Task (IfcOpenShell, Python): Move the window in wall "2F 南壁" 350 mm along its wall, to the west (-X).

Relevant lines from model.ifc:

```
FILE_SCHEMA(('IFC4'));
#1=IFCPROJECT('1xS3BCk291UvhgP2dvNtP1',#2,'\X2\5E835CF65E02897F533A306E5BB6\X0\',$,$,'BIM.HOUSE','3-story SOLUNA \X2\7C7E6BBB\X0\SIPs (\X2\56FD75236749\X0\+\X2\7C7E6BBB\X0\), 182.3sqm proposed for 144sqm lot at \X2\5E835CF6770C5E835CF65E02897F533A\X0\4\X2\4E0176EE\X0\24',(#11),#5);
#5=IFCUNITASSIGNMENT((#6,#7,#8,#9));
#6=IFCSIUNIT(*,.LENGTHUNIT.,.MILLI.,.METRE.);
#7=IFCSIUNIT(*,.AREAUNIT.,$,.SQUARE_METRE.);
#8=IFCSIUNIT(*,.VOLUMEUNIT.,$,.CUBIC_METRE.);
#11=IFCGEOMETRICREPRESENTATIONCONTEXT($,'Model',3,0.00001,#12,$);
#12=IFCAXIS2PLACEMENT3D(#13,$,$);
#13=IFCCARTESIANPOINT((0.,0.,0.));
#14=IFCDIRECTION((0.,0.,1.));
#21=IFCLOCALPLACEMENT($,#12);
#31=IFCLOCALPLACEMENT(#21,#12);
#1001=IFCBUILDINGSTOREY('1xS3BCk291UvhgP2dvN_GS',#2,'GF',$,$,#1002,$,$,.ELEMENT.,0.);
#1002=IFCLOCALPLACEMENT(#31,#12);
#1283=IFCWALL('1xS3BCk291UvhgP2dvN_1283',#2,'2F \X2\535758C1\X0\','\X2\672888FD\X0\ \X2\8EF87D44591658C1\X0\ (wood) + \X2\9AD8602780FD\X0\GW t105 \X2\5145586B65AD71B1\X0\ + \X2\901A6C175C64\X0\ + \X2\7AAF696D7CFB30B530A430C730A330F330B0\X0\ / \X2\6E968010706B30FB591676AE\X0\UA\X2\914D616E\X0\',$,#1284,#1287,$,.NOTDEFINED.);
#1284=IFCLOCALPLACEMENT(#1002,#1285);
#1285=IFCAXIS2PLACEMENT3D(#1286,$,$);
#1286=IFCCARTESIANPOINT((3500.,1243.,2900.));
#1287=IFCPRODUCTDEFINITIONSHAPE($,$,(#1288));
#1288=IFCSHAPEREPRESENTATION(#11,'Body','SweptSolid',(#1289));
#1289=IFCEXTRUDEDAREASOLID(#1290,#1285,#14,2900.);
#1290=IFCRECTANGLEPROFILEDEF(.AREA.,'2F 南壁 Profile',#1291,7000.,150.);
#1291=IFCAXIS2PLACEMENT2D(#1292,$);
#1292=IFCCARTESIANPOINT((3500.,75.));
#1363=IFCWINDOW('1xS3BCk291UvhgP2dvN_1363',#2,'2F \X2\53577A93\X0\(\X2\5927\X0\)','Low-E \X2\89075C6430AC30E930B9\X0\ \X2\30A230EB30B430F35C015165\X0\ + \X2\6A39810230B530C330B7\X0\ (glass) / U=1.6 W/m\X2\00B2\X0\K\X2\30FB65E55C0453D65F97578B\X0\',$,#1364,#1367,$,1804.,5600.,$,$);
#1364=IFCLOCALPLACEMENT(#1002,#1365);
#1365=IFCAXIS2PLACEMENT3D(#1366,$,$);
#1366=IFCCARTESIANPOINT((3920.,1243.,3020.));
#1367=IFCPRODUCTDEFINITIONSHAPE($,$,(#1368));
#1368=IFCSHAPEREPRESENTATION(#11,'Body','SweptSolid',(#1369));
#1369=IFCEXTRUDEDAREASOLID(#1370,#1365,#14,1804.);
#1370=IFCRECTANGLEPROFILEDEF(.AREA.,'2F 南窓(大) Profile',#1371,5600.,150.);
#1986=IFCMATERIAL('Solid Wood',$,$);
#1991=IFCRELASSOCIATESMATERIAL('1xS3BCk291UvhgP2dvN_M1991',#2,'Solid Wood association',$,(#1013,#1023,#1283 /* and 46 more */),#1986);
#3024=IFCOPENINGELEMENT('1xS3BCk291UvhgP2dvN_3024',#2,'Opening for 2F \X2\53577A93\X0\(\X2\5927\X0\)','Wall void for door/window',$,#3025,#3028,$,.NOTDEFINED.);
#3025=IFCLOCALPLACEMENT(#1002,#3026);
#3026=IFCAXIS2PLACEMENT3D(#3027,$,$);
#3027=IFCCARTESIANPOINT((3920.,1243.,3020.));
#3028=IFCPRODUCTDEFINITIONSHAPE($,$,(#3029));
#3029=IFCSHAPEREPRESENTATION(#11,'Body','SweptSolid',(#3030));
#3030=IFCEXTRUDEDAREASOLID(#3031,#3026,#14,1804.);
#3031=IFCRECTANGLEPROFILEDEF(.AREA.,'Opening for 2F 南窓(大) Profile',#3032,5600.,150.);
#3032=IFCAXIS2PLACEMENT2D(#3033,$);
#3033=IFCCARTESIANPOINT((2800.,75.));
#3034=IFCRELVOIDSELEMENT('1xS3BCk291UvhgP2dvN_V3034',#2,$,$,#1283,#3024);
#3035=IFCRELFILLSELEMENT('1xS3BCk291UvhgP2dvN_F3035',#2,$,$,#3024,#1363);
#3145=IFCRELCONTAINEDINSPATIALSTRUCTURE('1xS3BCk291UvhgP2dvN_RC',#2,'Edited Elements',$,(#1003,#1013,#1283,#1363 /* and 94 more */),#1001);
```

```python
import ifcopenshell
import ifcopenshell.api.geometry
import ifcopenshell.util.placement
import ifcopenshell.util.unit

model = ifcopenshell.open("model.ifc")
unit_scale = ifcopenshell.util.unit.calculate_unit_scale(model)

window = model.by_guid("1xS3BCk291UvhgP2dvN_1363")
opening = window.FillsVoids[0].RelatingOpeningElement
wall = opening.VoidsElements[0].RelatingBuildingElement

wall_matrix = ifcopenshell.util.placement.get_local_placement(wall.ObjectPlacement)
shift = wall_matrix[:3, 0] * -0.35 / unit_scale
before = ifcopenshell.util.placement.get_local_placement(window.ObjectPlacement)[:3, 3].copy()

# The window is not placed relative to its opening, so move both.
for product in (opening, window):
    matrix = ifcopenshell.util.placement.get_local_placement(product.ObjectPlacement)
    matrix[:3, 3] += shift
    ifcopenshell.api.geometry.edit_object_placement(model, product=product, matrix=matrix, is_si=False)

after = ifcopenshell.util.placement.get_local_placement(window.ObjectPlacement)[:3, 3]
print("window moved by", (after - before).round(3) + 0.0)

model.write("model_v2.ifc")
```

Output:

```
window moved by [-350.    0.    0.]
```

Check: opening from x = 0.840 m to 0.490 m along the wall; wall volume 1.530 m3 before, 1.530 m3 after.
